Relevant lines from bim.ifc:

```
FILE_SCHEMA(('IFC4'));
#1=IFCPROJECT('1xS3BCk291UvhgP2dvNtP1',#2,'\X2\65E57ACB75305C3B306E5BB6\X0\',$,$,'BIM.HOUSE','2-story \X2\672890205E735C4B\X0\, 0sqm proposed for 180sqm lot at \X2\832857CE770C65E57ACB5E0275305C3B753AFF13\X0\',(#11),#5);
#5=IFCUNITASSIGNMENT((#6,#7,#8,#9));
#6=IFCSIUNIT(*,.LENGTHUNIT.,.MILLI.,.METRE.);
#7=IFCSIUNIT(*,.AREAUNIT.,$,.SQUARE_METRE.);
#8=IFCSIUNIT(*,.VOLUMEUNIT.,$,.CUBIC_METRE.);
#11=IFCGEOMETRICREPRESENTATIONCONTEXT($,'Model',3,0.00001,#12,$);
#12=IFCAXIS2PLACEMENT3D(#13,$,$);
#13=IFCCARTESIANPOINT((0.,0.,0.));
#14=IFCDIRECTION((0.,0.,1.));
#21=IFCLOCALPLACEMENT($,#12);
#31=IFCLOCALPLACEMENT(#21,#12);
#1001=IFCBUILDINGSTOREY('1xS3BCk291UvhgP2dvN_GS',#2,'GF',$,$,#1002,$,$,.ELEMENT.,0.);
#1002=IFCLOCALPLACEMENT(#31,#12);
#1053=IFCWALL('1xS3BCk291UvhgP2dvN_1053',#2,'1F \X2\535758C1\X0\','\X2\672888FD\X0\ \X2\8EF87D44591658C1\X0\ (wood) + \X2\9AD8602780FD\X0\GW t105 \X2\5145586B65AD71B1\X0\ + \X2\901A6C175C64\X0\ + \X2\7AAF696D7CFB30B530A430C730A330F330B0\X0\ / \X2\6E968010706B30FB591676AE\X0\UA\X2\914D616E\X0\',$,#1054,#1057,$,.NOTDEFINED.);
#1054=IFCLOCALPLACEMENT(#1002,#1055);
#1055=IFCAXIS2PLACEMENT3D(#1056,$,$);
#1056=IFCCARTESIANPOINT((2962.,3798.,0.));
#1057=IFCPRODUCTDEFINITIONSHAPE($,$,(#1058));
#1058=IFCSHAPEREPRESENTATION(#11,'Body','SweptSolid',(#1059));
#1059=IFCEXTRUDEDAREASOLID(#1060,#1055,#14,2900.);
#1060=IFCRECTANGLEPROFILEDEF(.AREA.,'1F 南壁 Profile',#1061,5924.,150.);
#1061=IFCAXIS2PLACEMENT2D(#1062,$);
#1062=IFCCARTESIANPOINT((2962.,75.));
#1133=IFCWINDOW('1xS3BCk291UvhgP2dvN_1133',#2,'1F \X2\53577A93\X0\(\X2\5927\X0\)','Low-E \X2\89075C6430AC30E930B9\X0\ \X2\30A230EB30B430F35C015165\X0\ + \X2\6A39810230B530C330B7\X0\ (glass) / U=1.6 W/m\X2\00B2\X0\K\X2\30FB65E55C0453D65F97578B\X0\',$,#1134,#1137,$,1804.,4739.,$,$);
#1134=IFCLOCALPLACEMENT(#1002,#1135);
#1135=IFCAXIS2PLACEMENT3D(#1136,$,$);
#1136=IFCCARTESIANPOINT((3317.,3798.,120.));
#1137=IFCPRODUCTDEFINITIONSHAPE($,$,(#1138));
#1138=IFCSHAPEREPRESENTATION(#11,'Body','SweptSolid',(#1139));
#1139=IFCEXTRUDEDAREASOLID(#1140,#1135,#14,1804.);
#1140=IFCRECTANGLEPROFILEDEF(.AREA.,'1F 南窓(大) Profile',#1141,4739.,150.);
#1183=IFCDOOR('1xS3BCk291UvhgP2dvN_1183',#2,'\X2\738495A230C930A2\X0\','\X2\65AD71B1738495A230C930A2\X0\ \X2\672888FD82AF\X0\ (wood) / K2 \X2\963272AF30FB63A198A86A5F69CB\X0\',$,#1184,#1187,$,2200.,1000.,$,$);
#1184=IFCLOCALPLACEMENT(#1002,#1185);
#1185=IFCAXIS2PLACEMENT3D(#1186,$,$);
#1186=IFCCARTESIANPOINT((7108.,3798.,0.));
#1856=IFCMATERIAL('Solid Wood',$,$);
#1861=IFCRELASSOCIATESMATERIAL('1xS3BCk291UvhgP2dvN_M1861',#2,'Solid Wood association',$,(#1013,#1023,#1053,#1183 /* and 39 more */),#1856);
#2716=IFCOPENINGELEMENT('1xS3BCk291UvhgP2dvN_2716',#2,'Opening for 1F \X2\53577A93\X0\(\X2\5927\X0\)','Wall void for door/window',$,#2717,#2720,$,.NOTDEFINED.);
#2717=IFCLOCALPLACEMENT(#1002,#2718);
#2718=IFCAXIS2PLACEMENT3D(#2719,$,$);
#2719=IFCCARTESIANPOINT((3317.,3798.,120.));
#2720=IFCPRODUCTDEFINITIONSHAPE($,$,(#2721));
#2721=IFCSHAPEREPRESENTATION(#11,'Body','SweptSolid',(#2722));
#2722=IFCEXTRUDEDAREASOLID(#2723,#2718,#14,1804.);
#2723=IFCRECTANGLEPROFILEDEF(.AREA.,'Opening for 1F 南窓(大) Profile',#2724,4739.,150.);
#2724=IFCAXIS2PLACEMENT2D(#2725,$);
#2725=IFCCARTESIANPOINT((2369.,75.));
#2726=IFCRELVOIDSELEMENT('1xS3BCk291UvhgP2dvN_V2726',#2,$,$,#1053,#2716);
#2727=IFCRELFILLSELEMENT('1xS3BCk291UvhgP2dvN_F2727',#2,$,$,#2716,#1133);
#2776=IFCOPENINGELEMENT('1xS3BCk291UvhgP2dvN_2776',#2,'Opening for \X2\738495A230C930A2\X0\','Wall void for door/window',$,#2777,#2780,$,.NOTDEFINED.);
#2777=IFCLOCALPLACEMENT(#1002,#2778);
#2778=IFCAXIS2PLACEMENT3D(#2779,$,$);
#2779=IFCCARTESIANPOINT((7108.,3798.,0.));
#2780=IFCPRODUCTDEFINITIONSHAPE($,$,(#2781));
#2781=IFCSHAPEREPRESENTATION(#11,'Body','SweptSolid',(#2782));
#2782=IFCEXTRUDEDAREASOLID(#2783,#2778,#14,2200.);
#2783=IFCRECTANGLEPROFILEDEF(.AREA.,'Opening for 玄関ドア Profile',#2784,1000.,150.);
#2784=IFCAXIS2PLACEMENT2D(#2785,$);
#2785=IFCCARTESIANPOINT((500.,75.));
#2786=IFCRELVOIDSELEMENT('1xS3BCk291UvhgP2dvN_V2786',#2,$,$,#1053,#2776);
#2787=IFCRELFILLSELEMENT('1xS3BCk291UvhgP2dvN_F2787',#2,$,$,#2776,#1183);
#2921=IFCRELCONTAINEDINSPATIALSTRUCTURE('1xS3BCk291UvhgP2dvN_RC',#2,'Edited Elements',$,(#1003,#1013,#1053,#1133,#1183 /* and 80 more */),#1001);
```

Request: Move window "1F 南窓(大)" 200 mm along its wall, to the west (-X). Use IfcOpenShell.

```python
import ifcopenshell
import ifcopenshell.api.geometry
import ifcopenshell.util.placement
import ifcopenshell.util.unit

model = ifcopenshell.open("bim.ifc")
unit_scale = ifcopenshell.util.unit.calculate_unit_scale(model)

window = model.by_id(1133)
opening = window.FillsVoids[0].RelatingOpeningElement
wall = opening.VoidsElements[0].RelatingBuildingElement

wall_matrix = ifcopenshell.util.placement.get_local_placement(wall.ObjectPlacement)
shift = wall_matrix[:3, 0] * -0.2 / unit_scale
before = ifcopenshell.util.placement.get_local_placement(window.ObjectPlacement)[:3, 3].copy()

# The window is not placed relative to its opening, so move both.
for product in (opening, window):
    matrix = ifcopenshell.util.placement.get_local_placement(product.ObjectPlacement)
    matrix[:3, 3] += shift
    ifcopenshell.api.geometry.edit_object_placement(model, product=product, matrix=matrix, is_si=False)

after = ifcopenshell.util.placement.get_local_placement(window.ObjectPlacement)[:3, 3]
print("window moved by", (after - before).round(3) + 0.0)

model.write("bim-out.ifc")
```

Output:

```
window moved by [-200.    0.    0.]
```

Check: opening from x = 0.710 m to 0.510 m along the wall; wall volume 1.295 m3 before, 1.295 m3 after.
